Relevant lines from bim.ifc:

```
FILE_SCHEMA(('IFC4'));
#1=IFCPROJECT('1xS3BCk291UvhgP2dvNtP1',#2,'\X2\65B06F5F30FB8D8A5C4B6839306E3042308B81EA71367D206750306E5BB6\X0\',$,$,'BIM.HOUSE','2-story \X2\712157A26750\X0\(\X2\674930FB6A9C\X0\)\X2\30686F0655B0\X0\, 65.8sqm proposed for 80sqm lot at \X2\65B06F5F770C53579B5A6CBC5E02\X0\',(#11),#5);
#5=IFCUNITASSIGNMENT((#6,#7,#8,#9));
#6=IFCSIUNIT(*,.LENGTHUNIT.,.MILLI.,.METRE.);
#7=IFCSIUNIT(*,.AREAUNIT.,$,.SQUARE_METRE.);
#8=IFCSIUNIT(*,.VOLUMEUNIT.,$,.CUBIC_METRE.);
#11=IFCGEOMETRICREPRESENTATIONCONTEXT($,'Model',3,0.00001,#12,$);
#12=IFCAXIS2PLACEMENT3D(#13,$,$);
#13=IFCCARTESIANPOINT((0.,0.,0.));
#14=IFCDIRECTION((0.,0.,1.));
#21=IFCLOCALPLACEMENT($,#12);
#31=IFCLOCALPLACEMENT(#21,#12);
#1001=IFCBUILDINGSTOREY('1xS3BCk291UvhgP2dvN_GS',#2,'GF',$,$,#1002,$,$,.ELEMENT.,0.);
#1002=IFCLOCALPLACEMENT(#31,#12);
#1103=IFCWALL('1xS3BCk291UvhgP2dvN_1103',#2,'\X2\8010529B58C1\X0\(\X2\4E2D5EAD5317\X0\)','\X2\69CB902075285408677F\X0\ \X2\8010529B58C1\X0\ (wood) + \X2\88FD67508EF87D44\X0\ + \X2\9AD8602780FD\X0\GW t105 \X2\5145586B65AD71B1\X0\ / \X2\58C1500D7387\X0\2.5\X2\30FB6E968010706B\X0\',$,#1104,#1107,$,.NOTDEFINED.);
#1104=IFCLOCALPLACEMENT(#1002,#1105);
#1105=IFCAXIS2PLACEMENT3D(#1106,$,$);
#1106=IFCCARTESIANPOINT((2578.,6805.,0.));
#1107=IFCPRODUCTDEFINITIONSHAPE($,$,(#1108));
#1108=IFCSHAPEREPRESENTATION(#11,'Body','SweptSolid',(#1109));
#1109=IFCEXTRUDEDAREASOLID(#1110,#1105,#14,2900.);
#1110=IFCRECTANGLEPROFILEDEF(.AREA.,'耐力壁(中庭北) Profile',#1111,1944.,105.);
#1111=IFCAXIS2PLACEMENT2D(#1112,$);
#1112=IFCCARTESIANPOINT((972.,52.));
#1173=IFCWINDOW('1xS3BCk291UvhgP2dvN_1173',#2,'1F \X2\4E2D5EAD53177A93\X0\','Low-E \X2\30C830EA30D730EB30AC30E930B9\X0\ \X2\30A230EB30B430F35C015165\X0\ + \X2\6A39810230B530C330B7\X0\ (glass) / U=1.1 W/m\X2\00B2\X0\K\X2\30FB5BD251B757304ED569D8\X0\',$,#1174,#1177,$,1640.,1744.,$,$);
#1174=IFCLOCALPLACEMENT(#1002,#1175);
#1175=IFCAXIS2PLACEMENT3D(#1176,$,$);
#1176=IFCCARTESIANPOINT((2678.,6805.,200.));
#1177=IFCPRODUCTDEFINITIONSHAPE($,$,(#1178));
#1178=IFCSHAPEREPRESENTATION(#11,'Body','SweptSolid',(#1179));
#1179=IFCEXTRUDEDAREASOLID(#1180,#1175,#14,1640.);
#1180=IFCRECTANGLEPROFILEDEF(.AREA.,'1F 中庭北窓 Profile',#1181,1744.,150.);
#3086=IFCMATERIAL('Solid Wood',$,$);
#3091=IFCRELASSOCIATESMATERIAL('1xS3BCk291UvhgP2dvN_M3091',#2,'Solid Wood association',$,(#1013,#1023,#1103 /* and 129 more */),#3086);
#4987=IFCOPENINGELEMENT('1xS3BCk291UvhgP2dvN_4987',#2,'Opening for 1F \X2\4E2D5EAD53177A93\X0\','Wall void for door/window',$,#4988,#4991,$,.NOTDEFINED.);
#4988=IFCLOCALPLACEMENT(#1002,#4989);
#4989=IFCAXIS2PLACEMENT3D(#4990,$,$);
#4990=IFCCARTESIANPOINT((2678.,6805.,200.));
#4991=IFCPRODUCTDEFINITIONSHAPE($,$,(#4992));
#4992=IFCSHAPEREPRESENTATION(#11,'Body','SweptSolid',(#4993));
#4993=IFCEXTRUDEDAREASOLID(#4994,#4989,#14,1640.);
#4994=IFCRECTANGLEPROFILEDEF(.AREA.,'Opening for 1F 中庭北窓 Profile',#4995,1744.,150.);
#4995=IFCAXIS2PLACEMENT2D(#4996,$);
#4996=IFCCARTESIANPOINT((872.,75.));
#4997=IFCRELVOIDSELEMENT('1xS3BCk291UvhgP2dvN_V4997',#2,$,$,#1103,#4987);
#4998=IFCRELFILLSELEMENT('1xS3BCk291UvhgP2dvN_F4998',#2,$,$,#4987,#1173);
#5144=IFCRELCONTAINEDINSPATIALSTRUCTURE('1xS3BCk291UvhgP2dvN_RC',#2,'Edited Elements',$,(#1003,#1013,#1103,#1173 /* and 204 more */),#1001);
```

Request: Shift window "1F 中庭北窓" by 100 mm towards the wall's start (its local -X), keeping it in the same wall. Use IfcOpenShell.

```python
import ifcopenshell
import ifcopenshell.api.geometry
import ifcopenshell.util.placement
import ifcopenshell.util.unit

model = ifcopenshell.open("bim.ifc")
unit_scale = ifcopenshell.util.unit.calculate_unit_scale(model)

window = model.by_id(1173)
opening = window.FillsVoids[0].RelatingOpeningElement
wall = opening.VoidsElements[0].RelatingBuildingElement

wall_matrix = ifcopenshell.util.placement.get_local_placement(wall.ObjectPlacement)
shift = wall_matrix[:3, 0] * -0.1 / unit_scale
before = ifcopenshell.util.placement.get_local_placement(window.ObjectPlacement)[:3, 3].copy()

# The window is not placed relative to its opening, so move both.
for product in (opening, window):
    matrix = ifcopenshell.util.placement.get_local_placement(product.ObjectPlacement)
    matrix[:3, 3] += shift
    ifcopenshell.api.geometry.edit_object_placement(model, product=product, matrix=matrix, is_si=False)

after = ifcopenshell.util.placement.get_local_placement(window.ObjectPlacement)[:3, 3]
print("window moved by", (after - before).round(3) + 0.0)

model.write("bim_v2.ifc")
```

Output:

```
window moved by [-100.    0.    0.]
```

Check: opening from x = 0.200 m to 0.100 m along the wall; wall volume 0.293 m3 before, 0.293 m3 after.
